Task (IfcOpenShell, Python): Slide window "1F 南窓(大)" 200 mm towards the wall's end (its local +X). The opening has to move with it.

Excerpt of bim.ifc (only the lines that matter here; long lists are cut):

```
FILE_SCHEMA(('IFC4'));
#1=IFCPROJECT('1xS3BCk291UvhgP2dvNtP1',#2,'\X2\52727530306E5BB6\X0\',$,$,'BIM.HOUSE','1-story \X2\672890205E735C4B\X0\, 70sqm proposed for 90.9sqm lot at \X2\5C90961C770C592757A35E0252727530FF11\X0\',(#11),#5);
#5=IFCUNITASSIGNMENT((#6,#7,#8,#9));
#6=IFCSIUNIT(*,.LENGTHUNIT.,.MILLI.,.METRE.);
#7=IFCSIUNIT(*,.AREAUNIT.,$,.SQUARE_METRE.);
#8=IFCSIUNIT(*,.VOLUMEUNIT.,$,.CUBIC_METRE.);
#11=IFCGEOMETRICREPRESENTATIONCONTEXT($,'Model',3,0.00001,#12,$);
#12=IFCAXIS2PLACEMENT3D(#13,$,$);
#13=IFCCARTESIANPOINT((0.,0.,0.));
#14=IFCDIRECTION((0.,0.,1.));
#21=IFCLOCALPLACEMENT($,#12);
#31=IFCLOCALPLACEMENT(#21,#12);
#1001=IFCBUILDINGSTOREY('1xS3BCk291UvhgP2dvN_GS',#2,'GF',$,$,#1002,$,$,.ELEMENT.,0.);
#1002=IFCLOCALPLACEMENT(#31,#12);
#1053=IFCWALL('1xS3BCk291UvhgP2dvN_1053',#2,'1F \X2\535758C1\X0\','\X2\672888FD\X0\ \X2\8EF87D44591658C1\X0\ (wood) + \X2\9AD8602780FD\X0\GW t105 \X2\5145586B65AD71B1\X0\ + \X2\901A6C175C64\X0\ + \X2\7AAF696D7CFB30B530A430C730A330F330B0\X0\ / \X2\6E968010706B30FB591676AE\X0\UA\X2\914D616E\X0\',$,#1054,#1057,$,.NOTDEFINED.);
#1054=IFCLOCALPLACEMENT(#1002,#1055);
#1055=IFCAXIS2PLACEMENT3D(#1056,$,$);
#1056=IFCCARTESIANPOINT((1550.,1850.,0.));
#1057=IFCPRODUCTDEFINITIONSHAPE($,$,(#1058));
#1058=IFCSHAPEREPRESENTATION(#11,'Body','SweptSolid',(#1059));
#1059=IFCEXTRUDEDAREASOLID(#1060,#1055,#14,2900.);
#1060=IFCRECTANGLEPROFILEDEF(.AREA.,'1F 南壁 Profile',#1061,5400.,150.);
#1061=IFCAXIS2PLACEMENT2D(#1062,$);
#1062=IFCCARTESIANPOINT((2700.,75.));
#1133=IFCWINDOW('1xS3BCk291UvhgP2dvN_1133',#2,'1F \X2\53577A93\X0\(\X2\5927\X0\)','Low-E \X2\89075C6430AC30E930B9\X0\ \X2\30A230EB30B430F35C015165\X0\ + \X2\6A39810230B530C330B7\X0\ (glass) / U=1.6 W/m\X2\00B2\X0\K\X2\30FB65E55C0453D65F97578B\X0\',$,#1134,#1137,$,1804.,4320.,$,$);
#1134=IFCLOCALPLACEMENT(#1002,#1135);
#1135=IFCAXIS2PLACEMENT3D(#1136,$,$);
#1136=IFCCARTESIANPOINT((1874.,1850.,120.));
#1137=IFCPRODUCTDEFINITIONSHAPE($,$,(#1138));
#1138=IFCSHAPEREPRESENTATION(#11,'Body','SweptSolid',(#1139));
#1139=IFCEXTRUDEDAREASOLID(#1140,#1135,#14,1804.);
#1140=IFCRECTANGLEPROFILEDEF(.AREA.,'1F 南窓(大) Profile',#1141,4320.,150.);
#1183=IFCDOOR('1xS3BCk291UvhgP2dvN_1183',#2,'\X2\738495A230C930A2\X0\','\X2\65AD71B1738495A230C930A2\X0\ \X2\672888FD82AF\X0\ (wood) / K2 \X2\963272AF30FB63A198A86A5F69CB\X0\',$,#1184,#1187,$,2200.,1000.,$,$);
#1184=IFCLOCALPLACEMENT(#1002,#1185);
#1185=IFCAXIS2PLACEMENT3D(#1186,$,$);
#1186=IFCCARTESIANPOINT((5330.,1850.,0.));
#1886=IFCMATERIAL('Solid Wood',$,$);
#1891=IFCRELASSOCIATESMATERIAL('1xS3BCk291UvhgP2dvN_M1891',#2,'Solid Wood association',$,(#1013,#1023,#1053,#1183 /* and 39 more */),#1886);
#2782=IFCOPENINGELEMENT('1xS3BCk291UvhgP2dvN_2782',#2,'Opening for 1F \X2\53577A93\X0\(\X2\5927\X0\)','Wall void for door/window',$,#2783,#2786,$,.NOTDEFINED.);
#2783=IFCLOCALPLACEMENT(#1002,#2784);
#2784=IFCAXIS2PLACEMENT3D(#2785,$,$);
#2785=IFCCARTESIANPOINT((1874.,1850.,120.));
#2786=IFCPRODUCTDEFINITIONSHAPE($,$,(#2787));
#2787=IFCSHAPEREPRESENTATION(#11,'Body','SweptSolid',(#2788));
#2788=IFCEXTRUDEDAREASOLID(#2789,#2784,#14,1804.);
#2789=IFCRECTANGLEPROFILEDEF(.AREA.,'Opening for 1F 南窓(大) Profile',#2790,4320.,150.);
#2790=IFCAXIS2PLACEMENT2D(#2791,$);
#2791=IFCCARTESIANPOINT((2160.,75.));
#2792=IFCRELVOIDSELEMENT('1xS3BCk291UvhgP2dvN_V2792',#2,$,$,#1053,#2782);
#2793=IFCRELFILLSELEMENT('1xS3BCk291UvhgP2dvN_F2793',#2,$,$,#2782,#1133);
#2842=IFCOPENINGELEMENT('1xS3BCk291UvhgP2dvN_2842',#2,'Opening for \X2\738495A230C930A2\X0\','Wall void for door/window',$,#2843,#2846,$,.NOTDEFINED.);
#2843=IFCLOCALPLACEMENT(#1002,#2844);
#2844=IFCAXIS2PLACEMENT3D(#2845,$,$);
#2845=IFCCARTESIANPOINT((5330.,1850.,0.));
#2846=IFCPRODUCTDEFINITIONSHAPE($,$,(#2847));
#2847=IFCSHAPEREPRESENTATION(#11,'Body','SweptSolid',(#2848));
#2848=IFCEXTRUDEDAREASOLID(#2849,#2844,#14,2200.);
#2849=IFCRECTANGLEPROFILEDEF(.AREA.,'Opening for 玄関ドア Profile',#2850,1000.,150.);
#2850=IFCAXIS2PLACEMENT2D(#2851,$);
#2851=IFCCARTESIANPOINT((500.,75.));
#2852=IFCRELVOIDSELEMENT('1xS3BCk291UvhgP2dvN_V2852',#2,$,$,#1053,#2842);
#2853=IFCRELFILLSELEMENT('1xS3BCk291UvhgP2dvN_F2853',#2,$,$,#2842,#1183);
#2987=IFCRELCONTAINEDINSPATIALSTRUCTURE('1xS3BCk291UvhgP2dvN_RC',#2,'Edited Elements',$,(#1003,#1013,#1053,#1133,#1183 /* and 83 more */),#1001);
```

```python
import ifcopenshell
import ifcopenshell.api.geometry
import ifcopenshell.util.placement
import ifcopenshell.util.unit

model = ifcopenshell.open("bim.ifc")
unit_scale = ifcopenshell.util.unit.calculate_unit_scale(model)

window = model.by_guid("1xS3BCk291UvhgP2dvN_1133")
opening = window.FillsVoids[0].RelatingOpeningElement
wall = opening.VoidsElements[0].RelatingBuildingElement

wall_matrix = ifcopenshell.util.placement.get_local_placement(wall.ObjectPlacement)
shift = wall_matrix[:3, 0] * 0.2 / unit_scale
before = ifcopenshell.util.placement.get_local_placement(window.ObjectPlacement)[:3, 3].copy()

# The window is not placed relative to its opening, so move both.
for product in (opening, window):
    matrix = ifcopenshell.util.placement.get_local_placement(product.ObjectPlacement)
    matrix[:3, 3] += shift
    ifcopenshell.api.geometry.edit_object_placement(model, product=product, matrix=matrix, is_si=False)

after = ifcopenshell.util.placement.get_local_placement(window.ObjectPlacement)[:3, 3]
print("window moved by", (after - before).round(3) + 0.0)

model.write("bim_rev.ifc")
```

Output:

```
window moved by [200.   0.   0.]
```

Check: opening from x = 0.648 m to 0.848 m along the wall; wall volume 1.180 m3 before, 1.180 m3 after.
